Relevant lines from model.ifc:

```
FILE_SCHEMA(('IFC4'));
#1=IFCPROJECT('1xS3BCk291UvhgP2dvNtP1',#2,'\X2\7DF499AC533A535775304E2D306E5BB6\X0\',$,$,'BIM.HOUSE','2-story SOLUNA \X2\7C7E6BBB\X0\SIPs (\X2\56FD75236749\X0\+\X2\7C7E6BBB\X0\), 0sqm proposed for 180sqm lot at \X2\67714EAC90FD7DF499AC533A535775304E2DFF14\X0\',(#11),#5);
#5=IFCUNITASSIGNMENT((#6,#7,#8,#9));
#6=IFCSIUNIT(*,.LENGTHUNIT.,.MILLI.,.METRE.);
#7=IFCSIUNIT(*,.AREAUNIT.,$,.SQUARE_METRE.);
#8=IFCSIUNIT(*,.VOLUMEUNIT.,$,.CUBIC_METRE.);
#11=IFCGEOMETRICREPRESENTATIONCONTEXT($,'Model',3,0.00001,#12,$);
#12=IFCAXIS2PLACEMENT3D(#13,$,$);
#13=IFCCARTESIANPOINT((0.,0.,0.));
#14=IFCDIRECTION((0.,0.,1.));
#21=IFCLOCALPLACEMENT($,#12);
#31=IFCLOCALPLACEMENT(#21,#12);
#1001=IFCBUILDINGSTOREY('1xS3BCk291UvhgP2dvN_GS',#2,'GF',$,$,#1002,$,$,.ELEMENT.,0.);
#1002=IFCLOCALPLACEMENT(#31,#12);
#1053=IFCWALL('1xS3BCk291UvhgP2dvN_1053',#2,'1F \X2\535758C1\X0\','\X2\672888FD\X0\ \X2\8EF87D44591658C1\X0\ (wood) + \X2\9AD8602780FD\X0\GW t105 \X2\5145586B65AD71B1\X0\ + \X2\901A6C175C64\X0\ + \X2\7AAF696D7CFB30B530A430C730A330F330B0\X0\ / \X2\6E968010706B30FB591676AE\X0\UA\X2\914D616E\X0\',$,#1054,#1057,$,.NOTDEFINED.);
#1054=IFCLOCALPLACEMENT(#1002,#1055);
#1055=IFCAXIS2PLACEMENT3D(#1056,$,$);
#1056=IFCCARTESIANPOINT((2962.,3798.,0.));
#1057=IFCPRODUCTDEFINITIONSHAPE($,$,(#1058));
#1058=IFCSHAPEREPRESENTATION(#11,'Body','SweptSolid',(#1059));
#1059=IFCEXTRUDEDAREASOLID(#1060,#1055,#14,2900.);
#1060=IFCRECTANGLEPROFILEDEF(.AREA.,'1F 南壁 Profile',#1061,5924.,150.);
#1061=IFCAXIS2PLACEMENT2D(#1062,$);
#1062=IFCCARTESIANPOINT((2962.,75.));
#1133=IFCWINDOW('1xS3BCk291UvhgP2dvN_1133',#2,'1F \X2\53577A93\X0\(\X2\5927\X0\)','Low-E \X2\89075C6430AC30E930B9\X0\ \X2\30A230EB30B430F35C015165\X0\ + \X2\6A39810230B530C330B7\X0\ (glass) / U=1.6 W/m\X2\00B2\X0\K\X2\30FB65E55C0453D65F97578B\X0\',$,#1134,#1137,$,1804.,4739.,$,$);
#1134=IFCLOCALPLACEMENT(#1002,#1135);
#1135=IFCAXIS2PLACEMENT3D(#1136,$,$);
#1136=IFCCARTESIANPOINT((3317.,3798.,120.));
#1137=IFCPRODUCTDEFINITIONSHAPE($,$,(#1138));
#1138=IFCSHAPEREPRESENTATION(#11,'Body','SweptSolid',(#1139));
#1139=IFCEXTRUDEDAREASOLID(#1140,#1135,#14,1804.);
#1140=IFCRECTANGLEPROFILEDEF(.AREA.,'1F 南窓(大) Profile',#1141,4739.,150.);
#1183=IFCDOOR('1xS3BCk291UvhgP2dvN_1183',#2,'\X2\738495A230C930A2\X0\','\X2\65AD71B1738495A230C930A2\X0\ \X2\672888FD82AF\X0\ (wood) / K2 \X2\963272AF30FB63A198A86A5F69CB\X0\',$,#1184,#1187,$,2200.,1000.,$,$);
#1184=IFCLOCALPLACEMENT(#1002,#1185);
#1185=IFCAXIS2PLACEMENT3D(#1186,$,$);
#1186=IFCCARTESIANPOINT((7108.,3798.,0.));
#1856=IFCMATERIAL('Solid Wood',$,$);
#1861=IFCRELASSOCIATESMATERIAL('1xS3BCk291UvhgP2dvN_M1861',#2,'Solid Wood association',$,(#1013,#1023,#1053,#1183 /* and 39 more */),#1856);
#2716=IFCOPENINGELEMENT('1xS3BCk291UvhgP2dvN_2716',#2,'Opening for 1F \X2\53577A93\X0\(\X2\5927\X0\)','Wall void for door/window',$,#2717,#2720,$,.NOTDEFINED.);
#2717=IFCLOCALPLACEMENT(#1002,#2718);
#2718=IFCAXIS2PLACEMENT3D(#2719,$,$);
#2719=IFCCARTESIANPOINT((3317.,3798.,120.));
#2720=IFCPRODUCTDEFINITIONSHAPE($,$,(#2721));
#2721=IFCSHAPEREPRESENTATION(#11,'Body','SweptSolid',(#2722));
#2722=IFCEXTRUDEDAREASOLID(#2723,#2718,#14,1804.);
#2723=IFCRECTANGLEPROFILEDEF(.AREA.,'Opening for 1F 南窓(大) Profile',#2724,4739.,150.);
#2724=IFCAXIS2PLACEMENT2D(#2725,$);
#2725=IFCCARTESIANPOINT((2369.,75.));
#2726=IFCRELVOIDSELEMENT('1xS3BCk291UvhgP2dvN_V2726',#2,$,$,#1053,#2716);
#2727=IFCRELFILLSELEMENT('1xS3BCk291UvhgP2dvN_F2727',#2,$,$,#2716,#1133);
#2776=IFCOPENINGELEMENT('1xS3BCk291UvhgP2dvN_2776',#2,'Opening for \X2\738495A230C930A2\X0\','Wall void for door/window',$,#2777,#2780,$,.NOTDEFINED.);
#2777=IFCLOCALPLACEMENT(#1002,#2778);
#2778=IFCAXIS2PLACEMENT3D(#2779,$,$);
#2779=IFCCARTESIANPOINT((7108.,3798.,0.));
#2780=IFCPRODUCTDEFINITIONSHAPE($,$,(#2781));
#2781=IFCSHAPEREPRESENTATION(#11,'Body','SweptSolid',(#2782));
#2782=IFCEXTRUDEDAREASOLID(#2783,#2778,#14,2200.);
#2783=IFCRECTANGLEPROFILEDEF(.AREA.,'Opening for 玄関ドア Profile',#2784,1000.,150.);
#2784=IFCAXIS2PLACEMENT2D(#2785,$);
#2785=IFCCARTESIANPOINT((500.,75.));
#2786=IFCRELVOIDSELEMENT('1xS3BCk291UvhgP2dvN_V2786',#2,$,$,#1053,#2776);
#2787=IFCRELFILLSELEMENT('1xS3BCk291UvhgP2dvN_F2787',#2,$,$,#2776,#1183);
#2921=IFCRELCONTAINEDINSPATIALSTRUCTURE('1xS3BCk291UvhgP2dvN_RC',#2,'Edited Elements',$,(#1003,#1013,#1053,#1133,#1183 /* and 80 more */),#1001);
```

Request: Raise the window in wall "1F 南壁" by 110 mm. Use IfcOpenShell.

```python
import numpy as np
import ifcopenshell
import ifcopenshell.api.geometry
import ifcopenshell.util.placement
import ifcopenshell.util.unit

model = ifcopenshell.open("model.ifc")
unit_scale = ifcopenshell.util.unit.calculate_unit_scale(model)

window = model.by_guid("1xS3BCk291UvhgP2dvN_1133")
opening = window.FillsVoids[0].RelatingOpeningElement
dz = 110.0

shift = np.array([0.0, 0.0, dz])
# The window is not placed relative to its opening, so move both.
for product in (opening, window):
    matrix = ifcopenshell.util.placement.get_local_placement(product.ObjectPlacement)
    matrix[:3, 3] += shift
    ifcopenshell.api.geometry.edit_object_placement(model, product=product, matrix=matrix, is_si=False)

print(f"moved by {dz * unit_scale:+.3f} m")

model.write("model_rev.ifc")
```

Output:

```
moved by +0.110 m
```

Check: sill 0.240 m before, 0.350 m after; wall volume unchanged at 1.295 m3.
